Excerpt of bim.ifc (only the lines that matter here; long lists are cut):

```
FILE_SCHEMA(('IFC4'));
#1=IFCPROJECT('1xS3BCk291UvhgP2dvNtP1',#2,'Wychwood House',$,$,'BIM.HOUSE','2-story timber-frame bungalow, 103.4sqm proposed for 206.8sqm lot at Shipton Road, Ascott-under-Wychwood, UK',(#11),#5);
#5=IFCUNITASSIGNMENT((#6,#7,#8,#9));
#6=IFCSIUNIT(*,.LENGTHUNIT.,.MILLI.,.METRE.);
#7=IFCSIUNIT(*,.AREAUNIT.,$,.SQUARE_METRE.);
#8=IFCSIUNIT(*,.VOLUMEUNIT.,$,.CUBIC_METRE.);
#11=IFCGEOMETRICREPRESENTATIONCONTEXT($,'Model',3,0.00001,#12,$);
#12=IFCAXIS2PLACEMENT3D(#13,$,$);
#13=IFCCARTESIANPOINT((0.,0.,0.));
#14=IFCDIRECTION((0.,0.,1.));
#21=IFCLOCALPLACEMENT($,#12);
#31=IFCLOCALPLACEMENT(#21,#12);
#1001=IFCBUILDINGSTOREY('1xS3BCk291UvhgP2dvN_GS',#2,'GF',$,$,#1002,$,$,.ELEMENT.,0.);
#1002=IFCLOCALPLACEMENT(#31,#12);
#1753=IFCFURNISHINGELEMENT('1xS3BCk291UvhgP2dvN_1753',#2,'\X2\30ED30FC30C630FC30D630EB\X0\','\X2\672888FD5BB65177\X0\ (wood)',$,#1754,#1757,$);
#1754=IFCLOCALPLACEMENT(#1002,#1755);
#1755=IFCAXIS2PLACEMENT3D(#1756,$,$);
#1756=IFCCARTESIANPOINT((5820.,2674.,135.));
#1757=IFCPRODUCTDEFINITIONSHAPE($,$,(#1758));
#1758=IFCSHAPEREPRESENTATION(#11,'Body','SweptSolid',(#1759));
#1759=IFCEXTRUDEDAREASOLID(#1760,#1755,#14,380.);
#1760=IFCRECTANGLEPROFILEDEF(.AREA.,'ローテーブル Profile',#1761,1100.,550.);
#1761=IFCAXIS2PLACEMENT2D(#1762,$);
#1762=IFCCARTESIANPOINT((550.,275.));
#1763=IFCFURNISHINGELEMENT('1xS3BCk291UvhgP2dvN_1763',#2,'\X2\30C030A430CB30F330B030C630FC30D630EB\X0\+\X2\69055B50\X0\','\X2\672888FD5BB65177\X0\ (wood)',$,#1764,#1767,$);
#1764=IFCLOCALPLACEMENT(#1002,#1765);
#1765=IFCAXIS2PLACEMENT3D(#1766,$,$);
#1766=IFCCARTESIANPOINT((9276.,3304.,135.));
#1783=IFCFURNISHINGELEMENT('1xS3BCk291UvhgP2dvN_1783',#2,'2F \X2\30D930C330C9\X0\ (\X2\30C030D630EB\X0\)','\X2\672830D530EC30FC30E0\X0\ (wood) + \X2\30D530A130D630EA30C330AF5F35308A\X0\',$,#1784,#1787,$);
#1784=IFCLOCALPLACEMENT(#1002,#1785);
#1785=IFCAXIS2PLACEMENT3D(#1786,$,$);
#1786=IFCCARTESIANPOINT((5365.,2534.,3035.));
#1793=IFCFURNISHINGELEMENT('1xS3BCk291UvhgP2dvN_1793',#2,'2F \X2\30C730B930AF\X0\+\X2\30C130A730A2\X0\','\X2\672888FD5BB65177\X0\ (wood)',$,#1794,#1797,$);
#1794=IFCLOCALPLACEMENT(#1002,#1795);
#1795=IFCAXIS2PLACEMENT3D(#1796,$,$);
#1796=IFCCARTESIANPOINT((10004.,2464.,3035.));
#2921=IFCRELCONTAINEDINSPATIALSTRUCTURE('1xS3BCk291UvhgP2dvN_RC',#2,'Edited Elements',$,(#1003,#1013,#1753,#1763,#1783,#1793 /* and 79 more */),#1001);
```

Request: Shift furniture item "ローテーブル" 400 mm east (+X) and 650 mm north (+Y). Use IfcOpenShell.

```python
import ifcopenshell
import ifcopenshell.api.geometry
import ifcopenshell.util.placement

model = ifcopenshell.open("bim.ifc")

item = model.by_guid("1xS3BCk291UvhgP2dvN_1753")
matrix = ifcopenshell.util.placement.get_local_placement(item.ObjectPlacement)
matrix[0, 3] += 400.0
matrix[1, 3] += 650.0
ifcopenshell.api.geometry.edit_object_placement(model, product=item, matrix=matrix, is_si=False)

print(ifcopenshell.util.placement.get_local_placement(item.ObjectPlacement).round(3) + 0.0)

model.write("bim_rev.ifc")
```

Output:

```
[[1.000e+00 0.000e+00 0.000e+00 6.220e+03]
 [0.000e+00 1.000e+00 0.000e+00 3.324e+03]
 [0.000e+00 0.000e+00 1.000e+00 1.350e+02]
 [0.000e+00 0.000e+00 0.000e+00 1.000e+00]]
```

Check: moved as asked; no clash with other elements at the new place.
